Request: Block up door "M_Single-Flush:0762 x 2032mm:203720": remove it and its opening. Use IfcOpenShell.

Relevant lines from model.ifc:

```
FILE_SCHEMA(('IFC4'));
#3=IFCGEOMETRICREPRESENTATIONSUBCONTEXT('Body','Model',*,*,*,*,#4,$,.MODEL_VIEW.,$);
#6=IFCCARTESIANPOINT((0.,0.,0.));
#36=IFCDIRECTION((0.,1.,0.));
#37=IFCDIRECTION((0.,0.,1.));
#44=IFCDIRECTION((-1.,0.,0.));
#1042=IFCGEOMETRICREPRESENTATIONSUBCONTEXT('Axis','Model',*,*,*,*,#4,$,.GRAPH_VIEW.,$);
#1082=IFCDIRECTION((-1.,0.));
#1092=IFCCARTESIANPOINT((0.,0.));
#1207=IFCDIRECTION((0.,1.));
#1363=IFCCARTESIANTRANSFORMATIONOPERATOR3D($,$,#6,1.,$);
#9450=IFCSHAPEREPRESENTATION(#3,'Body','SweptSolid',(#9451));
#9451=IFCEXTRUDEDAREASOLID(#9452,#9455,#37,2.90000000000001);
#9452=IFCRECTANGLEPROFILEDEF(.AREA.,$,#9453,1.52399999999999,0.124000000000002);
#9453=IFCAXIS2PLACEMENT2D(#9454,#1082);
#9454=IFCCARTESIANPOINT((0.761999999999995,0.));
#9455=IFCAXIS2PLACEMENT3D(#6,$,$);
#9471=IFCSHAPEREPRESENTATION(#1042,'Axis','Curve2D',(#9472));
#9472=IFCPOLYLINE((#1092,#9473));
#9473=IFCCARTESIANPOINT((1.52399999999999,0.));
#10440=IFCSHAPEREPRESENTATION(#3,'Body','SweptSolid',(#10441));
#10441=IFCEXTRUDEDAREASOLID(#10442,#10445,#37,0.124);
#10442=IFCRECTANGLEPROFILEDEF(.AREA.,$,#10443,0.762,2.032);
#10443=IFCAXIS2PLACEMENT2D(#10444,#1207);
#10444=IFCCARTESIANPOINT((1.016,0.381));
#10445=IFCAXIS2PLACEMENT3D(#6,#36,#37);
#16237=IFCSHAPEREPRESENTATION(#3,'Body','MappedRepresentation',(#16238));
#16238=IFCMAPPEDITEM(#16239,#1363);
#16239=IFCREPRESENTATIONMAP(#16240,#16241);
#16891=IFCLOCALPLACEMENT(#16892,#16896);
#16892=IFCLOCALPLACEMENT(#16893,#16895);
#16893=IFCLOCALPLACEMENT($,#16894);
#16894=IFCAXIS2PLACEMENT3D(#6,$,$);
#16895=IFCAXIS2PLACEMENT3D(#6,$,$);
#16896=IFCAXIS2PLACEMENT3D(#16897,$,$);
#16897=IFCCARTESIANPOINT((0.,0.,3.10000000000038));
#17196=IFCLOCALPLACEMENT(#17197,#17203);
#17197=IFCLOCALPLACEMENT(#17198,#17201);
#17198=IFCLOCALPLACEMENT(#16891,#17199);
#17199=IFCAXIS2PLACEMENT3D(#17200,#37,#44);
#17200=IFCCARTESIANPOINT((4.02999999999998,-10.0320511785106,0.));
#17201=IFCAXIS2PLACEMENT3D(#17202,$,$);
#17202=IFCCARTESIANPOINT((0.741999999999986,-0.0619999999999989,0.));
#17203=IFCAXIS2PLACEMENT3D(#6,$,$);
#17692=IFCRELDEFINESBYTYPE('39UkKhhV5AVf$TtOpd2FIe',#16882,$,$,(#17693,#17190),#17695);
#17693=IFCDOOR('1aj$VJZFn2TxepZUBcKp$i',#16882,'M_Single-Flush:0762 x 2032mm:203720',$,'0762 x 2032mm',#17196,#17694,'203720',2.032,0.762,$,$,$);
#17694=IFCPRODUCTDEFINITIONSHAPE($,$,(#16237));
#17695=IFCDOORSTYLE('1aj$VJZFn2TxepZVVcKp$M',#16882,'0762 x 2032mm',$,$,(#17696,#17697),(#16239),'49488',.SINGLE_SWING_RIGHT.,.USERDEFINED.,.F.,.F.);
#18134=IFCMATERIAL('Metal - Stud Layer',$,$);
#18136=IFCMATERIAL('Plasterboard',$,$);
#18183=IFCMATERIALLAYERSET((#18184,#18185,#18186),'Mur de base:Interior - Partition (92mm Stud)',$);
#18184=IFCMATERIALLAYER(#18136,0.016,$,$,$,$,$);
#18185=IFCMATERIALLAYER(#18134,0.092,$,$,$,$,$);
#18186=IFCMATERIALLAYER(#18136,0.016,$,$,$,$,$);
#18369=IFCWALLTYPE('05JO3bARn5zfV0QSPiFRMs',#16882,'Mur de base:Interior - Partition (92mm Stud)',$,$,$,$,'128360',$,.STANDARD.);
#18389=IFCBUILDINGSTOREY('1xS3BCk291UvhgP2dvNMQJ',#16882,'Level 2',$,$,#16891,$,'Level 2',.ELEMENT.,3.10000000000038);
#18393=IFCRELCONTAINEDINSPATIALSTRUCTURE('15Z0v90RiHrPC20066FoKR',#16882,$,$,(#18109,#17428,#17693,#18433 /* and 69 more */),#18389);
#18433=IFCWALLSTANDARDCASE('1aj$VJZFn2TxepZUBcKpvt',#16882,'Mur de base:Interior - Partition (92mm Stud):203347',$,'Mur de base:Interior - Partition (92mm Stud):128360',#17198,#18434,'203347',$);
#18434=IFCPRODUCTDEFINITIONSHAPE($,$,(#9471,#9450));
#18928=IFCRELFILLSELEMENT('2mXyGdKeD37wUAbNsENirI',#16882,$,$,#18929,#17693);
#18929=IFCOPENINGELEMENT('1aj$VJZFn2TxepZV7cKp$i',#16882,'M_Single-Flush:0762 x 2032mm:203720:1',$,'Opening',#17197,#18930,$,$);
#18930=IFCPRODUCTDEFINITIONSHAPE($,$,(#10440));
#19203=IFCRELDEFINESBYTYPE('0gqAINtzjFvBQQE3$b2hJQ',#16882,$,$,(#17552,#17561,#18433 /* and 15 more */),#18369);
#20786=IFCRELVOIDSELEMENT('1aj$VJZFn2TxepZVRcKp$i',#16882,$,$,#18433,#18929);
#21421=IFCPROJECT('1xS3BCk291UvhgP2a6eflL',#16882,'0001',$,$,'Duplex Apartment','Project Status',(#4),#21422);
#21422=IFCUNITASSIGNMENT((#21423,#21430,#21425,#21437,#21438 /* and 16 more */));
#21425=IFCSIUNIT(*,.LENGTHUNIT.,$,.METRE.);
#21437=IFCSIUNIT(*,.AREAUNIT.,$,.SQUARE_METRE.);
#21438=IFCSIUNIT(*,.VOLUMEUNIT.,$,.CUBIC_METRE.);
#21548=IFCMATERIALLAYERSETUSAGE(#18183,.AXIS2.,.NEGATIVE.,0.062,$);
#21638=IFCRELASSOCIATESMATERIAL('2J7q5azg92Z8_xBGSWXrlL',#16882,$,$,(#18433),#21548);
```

```python
import ifcopenshell
import ifcopenshell.api.feature
import ifcopenshell.api.root
import ifcopenshell.geom
import ifcopenshell.util.shape

model = ifcopenshell.open("model.ifc")
settings = ifcopenshell.geom.settings()


def volume(element):
    """Net volume in cubic metres, openings subtracted."""
    shape = ifcopenshell.geom.create_shape(settings, element)
    return ifcopenshell.util.shape.get_volume(shape.geometry)


door = model.by_guid("1aj$VJZFn2TxepZUBcKp$i")
opening = door.FillsVoids[0].RelatingOpeningElement
wall = opening.VoidsElements[0].RelatingBuildingElement
before = volume(wall)

ifcopenshell.api.root.remove_product(model, product=door)
ifcopenshell.api.feature.remove_feature(model, feature=opening)

after = volume(wall)

print(f"wall volume {before:.3f} -> {after:.3f} m3")

model.write("model_edited.ifc")
```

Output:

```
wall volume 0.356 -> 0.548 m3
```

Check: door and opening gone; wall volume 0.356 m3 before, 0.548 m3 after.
